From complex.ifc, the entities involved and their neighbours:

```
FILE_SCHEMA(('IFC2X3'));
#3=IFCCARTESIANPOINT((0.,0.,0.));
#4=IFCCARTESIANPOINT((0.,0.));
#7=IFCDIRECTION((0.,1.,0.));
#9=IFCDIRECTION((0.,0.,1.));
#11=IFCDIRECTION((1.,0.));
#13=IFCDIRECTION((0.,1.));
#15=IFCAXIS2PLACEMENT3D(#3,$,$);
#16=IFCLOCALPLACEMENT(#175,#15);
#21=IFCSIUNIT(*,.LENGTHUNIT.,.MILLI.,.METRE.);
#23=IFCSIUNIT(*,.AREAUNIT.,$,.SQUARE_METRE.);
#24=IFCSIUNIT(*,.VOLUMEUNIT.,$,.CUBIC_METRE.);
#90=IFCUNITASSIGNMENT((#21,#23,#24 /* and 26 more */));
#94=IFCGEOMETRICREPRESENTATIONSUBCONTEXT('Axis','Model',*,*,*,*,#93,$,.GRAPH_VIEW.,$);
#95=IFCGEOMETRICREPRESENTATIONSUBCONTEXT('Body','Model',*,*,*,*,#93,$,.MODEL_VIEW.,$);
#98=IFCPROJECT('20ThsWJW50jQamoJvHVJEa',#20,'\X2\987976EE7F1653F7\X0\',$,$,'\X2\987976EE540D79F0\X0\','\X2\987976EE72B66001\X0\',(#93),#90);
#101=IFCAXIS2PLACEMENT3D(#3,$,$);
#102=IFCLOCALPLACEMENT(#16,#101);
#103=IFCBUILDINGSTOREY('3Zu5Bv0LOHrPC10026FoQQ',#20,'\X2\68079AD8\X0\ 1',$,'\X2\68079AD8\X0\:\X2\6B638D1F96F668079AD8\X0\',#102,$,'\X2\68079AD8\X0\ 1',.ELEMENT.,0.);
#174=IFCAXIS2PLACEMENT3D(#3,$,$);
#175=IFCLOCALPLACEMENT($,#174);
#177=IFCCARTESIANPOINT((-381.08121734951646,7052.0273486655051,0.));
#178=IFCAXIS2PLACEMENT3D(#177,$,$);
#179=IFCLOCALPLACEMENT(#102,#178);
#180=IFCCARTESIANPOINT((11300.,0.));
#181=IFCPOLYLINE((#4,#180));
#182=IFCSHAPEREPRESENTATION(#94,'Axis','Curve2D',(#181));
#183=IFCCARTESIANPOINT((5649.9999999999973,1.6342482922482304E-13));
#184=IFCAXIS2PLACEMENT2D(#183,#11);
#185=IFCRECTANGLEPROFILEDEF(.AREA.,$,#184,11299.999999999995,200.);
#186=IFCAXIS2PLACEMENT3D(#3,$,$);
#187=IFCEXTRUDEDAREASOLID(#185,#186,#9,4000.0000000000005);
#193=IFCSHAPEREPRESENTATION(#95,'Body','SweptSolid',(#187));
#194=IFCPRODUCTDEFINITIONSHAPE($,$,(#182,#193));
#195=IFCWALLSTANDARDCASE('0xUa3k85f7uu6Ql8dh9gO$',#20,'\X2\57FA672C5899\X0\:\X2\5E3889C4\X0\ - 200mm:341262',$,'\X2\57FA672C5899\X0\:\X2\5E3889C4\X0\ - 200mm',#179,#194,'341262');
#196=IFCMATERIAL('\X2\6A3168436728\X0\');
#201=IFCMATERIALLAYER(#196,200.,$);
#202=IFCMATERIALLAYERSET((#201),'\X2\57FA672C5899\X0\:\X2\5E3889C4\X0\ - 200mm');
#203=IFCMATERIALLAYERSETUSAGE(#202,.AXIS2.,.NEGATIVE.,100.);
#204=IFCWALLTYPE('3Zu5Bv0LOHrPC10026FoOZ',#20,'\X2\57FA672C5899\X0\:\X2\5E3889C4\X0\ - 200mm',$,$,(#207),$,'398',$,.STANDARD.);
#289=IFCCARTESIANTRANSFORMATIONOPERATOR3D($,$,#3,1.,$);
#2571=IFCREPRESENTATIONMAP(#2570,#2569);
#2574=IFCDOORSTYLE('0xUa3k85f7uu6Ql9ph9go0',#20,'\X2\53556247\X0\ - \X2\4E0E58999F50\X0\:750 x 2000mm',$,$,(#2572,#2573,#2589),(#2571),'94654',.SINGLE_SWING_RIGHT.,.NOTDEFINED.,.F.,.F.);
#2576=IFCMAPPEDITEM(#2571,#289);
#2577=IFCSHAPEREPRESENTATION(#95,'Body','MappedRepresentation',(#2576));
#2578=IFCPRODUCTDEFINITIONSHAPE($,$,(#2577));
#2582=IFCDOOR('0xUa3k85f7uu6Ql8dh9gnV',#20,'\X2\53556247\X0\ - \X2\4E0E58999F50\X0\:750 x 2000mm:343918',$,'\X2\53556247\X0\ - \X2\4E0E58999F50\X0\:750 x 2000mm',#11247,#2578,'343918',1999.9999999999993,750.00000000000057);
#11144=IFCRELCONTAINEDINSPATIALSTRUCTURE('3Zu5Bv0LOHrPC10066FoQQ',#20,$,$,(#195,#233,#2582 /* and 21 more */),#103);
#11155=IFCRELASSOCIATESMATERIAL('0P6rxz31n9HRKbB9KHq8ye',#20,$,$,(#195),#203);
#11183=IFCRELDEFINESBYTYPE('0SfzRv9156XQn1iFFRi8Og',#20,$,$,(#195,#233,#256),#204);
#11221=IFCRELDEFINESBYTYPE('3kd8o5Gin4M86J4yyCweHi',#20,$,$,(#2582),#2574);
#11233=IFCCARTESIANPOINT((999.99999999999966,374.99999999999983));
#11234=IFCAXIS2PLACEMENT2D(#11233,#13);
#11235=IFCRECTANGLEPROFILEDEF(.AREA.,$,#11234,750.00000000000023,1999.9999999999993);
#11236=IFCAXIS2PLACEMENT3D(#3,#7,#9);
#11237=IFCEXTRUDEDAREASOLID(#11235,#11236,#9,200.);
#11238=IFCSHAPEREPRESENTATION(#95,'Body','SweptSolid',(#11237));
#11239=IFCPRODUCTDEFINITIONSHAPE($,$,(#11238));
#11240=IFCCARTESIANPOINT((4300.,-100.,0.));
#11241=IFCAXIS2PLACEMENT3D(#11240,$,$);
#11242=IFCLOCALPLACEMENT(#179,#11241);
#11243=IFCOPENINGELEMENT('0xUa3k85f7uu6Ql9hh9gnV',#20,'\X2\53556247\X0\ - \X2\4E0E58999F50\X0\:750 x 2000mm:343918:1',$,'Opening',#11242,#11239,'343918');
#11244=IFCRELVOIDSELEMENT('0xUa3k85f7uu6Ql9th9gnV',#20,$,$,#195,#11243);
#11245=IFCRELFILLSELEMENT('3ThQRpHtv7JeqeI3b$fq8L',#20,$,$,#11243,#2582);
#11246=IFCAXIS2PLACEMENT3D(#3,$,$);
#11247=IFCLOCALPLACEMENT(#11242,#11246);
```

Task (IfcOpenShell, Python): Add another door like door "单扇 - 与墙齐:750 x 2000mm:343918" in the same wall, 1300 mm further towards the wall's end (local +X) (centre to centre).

```python
import ifcopenshell
import ifcopenshell.api.feature
import ifcopenshell.api.geometry
import ifcopenshell.api.root
import ifcopenshell.geom
import ifcopenshell.util.element
import ifcopenshell.util.placement
import ifcopenshell.util.shape
import ifcopenshell.util.unit

model = ifcopenshell.open("complex.ifc")
unit_scale = ifcopenshell.util.unit.calculate_unit_scale(model)
settings = ifcopenshell.geom.settings()


def volume(element):
    """Net volume in cubic metres, openings subtracted."""
    shape = ifcopenshell.geom.create_shape(settings, element)
    return ifcopenshell.util.shape.get_volume(shape.geometry)


def reuse_history(source, copy):
    """copy_class also copies each property set's owner history, people and application; keep the originals."""
    for rel in copy.IsDefinedBy:
        if rel.is_a("IfcRelDefinesByProperties") and (history := rel.RelatingPropertyDefinition.OwnerHistory):
            rel.RelatingPropertyDefinition.OwnerHistory = source.OwnerHistory
            ifcopenshell.util.element.remove_deep2(model, history)


door = model.by_id(2582)
opening = door.FillsVoids[0].RelatingOpeningElement
wall = opening.VoidsElements[0].RelatingBuildingElement
before = volume(wall)
shift = ifcopenshell.util.placement.get_local_placement(wall.ObjectPlacement)[:3, 0] * 1.3 / unit_scale

# copy_class copies the void relationship, type, container and properties, but no geometry.
new_opening = ifcopenshell.api.root.copy_class(model, product=opening)
new_opening.Representation = ifcopenshell.util.element.copy_deep(
    model, opening.Representation, exclude=["IfcGeometricRepresentationContext", "IfcRepresentationMap"]
)
new_opening.Name = "单扇 - 与墙齐:750 x 2000mm"
new_opening.Tag = None
new_door = ifcopenshell.api.root.copy_class(model, product=door)
new_door.Representation = ifcopenshell.util.element.copy_deep(
    model, door.Representation, exclude=["IfcGeometricRepresentationContext", "IfcRepresentationMap"]
)
new_door.Name = "单扇 - 与墙齐:750 x 2000mm"
new_door.Tag = None
reuse_history(door, new_door)
fills = ifcopenshell.api.feature.add_filling(model, opening=new_opening, element=new_door)
fills.OwnerHistory = new_door.OwnerHistory  # required in IFC2X3

for old, new in ((opening, new_opening), (door, new_door)):
    matrix = ifcopenshell.util.placement.get_local_placement(old.ObjectPlacement)
    matrix[:3, 3] += shift
    ifcopenshell.api.geometry.edit_object_placement(model, product=new, matrix=matrix, is_si=False)

after = volume(wall)

print(f"wall volume {before:.3f} -> {after:.3f} m3")

model.write("complex_updated.ifc")
```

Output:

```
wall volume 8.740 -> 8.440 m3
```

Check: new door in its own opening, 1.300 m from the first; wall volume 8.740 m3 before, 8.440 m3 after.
